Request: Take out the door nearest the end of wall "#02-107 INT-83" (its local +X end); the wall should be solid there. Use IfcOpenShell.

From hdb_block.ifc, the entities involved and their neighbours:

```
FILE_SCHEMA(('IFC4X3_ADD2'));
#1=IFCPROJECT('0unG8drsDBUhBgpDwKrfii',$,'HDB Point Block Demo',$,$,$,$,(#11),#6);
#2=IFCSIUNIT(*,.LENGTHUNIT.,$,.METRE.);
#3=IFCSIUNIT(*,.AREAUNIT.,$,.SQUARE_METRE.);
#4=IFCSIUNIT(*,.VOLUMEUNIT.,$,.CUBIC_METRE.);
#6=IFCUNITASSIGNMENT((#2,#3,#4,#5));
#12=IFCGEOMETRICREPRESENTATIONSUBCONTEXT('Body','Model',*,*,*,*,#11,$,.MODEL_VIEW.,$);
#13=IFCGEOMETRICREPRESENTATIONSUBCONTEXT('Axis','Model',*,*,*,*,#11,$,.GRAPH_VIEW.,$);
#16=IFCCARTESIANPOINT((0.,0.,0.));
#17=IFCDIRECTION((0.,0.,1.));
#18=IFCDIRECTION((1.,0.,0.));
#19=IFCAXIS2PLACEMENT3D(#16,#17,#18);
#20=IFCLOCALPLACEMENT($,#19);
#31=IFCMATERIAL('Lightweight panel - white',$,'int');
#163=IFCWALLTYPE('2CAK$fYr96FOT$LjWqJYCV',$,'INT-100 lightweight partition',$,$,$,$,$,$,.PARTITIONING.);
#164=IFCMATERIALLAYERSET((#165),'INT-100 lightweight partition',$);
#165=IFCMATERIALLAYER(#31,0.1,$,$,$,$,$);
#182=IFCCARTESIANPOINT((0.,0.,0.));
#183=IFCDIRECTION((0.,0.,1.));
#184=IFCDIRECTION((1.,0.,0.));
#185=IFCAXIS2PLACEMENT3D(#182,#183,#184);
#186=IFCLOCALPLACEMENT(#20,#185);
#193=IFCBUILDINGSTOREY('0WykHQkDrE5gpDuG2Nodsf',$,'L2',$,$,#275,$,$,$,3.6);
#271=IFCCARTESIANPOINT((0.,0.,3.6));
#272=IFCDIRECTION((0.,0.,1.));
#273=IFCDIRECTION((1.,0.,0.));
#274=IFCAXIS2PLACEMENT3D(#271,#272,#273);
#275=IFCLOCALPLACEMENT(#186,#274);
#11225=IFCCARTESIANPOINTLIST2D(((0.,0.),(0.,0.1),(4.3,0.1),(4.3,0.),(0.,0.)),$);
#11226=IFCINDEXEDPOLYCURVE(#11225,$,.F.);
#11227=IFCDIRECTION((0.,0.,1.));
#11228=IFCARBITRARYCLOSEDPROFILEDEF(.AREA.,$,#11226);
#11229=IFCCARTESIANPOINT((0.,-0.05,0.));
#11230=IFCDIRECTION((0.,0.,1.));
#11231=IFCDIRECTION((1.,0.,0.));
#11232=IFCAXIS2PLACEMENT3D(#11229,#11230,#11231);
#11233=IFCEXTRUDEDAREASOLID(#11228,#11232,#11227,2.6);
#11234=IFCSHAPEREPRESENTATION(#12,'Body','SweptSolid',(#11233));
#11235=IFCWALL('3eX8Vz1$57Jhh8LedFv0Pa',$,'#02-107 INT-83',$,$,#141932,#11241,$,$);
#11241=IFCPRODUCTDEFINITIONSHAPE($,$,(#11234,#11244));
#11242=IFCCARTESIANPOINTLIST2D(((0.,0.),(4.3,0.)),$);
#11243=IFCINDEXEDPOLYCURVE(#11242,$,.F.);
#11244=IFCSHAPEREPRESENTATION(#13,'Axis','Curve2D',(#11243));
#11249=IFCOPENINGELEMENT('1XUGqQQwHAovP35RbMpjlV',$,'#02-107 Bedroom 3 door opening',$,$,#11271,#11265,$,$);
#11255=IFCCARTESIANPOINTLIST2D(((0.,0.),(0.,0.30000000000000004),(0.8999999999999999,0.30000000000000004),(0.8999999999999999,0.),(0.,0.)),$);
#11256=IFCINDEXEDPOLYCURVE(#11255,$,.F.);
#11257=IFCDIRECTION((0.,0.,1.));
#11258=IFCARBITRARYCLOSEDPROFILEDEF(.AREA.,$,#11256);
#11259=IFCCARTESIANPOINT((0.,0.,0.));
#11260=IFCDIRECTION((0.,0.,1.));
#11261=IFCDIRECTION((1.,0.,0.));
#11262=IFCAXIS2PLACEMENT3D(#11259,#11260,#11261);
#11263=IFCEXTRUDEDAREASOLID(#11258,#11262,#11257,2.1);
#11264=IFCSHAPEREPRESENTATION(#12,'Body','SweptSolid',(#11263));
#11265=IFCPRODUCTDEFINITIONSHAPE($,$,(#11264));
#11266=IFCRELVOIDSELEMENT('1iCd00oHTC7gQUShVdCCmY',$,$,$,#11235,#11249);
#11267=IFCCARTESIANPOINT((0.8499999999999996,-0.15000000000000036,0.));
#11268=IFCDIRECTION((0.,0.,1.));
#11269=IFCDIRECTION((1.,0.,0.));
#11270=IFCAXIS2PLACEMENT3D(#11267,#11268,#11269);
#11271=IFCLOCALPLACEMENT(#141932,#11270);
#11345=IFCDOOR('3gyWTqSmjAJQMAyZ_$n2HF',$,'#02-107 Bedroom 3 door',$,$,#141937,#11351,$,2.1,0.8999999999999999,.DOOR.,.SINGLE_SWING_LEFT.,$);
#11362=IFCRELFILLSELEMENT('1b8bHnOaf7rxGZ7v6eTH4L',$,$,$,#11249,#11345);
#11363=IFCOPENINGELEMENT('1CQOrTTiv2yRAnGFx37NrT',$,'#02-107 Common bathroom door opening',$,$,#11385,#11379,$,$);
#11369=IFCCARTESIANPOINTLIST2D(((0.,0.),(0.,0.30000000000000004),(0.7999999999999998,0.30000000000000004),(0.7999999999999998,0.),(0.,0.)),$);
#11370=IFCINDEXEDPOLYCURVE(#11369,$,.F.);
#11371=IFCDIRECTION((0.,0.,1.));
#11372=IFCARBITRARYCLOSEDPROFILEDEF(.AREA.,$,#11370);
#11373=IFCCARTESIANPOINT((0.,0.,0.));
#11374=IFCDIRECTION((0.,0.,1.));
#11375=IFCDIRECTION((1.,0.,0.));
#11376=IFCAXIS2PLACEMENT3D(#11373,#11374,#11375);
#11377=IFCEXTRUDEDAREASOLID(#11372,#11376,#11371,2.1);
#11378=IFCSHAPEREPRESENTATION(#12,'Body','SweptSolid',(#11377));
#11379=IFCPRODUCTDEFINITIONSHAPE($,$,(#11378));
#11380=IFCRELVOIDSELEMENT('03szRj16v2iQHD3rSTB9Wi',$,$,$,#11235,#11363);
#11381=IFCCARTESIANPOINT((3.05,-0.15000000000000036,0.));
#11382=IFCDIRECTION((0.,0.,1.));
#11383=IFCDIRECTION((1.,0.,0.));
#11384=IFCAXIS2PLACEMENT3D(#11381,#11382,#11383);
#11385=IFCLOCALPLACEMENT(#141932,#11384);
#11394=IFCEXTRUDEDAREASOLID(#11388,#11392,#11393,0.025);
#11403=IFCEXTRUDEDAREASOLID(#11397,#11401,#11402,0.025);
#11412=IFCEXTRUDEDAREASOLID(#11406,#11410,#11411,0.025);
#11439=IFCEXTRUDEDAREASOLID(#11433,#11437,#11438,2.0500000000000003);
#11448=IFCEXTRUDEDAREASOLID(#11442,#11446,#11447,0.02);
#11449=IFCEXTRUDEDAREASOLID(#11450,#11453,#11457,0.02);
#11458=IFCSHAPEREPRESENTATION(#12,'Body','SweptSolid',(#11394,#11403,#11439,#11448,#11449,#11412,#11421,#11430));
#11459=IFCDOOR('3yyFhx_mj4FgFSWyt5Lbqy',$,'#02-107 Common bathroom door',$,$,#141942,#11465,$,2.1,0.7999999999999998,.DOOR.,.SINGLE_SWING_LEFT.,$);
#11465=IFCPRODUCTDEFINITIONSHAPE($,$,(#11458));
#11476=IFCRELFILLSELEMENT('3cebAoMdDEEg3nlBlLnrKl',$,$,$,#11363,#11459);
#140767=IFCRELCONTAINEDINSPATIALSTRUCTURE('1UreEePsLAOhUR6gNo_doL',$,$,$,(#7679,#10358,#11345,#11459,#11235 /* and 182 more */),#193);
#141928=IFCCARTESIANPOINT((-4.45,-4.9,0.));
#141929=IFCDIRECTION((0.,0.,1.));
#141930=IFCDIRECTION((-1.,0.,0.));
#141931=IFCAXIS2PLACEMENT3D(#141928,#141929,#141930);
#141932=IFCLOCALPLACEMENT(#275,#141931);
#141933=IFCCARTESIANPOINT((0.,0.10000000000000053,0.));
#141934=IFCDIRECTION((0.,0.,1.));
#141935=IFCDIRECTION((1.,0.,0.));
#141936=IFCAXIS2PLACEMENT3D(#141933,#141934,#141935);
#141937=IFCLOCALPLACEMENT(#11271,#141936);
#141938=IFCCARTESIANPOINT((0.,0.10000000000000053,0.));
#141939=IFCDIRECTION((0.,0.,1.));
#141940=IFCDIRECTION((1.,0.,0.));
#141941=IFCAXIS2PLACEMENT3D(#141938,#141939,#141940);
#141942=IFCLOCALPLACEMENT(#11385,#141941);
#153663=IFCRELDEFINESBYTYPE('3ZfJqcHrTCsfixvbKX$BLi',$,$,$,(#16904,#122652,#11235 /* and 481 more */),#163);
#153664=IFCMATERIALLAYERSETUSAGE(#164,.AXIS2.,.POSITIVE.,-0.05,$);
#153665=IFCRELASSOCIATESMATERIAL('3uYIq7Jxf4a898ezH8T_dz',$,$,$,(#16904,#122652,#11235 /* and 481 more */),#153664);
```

```python
import ifcopenshell
import ifcopenshell.api.feature
import ifcopenshell.api.root
import ifcopenshell.geom
import ifcopenshell.util.shape

model = ifcopenshell.open("hdb_block.ifc")
settings = ifcopenshell.geom.settings()


def volume(element):
    """Net volume in cubic metres, openings subtracted."""
    shape = ifcopenshell.geom.create_shape(settings, element)
    return ifcopenshell.util.shape.get_volume(shape.geometry)


door = model.by_id(11459)
opening = door.FillsVoids[0].RelatingOpeningElement
wall = opening.VoidsElements[0].RelatingBuildingElement
before = volume(wall)

ifcopenshell.api.root.remove_product(model, product=door)
ifcopenshell.api.feature.remove_feature(model, feature=opening)

after = volume(wall)

print(f"wall volume {before:.3f} -> {after:.3f} m3")

model.write("hdb_block-out.ifc")
```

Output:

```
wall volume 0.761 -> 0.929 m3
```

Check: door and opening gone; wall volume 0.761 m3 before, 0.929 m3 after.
